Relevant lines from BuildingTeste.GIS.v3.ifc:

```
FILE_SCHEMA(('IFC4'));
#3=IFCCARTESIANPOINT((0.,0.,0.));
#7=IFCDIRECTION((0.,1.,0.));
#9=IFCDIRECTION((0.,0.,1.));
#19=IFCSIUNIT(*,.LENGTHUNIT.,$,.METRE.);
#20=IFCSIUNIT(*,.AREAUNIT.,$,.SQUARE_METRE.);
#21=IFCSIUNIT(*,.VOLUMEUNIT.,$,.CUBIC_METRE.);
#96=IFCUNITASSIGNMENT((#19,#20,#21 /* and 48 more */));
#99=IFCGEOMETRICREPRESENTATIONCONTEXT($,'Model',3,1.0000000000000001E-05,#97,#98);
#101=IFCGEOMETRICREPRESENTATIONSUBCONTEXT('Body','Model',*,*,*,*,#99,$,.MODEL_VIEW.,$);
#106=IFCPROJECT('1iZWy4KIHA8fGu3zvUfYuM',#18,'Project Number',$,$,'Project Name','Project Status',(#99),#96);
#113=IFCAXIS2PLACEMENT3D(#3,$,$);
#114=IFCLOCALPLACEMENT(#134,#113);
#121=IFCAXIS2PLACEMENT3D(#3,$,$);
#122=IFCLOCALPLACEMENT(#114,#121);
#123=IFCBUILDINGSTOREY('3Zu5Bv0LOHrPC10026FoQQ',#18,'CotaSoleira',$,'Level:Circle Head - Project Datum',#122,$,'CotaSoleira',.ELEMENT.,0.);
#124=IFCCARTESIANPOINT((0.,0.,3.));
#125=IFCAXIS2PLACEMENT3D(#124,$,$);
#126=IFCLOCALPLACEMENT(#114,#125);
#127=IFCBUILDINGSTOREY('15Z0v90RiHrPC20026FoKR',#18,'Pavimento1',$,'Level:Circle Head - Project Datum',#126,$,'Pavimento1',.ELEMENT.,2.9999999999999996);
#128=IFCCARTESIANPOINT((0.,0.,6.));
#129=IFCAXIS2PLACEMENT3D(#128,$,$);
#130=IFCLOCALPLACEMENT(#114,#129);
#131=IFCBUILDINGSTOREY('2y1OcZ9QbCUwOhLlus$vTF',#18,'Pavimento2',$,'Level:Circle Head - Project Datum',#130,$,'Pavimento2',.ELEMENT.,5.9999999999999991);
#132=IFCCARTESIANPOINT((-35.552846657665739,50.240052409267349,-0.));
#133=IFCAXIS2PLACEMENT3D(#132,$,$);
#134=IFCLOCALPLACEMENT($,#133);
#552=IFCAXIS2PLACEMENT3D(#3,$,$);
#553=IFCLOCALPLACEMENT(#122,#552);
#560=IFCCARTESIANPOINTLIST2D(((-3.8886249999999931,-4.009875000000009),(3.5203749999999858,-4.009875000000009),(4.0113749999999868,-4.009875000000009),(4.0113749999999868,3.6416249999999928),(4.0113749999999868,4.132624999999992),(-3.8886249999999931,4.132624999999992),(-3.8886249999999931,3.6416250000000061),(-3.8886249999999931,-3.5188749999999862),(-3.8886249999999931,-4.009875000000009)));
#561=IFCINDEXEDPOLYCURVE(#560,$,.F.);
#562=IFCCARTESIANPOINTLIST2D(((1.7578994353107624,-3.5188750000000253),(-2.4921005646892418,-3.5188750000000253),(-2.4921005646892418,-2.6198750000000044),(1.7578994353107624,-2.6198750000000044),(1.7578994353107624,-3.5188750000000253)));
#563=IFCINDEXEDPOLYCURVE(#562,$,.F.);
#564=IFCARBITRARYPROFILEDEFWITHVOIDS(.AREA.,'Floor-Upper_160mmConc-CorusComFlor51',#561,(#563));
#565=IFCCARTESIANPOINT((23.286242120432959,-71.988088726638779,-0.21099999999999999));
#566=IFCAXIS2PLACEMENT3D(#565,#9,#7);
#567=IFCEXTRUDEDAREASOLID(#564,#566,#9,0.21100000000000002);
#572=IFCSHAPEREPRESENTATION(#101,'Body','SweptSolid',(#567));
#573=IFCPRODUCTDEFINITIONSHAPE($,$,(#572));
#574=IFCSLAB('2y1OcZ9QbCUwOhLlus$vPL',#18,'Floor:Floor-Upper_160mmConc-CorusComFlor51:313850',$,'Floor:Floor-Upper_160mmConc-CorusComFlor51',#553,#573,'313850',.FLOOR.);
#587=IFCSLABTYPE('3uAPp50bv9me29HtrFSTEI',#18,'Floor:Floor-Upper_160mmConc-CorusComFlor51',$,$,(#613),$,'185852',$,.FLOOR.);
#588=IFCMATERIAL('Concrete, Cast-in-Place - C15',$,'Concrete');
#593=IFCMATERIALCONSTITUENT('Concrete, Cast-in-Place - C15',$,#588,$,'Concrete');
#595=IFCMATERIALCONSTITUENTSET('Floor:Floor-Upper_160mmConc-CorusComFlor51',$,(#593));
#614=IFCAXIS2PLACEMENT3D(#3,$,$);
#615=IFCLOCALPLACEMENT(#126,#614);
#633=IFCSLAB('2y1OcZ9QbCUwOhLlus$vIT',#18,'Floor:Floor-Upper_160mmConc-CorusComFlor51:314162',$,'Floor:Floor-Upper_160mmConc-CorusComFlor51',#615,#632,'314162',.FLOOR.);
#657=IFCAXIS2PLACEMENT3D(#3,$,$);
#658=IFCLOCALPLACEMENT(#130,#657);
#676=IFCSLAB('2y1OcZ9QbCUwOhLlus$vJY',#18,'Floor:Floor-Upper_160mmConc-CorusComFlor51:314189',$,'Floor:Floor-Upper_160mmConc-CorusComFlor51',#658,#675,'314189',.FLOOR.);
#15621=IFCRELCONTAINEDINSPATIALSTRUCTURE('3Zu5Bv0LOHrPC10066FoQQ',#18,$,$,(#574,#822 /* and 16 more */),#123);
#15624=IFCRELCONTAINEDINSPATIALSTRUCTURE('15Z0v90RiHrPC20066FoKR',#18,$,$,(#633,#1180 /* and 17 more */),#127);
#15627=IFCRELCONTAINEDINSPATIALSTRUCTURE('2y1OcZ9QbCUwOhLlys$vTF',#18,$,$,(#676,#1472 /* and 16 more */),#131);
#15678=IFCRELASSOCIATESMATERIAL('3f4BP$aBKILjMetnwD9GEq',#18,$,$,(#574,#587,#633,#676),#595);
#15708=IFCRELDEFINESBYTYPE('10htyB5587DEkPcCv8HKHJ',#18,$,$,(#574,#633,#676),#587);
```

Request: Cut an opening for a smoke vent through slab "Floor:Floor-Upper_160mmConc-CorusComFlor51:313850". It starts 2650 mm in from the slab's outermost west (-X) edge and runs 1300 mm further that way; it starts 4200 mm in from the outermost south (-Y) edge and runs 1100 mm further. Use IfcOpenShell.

```python
import numpy as np
import ifcopenshell
import ifcopenshell.api.feature
import ifcopenshell.api.geometry
import ifcopenshell.api.root
import ifcopenshell.geom
import ifcopenshell.util.placement
import ifcopenshell.util.representation
import ifcopenshell.util.shape
import ifcopenshell.util.unit

model = ifcopenshell.open("BuildingTeste.GIS.v3.ifc")
unit_scale = ifcopenshell.util.unit.calculate_unit_scale(model)
settings = ifcopenshell.geom.settings()


def volume(element):
    """Net volume in cubic metres, openings subtracted."""
    shape = ifcopenshell.geom.create_shape(settings, element)
    return ifcopenshell.util.shape.get_volume(shape.geometry)


slab = model.by_id(574)
before = volume(slab)

# Extent in the slab's own axes, in metres. The edges named are its -X and -Y sides.
slab_shape = ifcopenshell.geom.create_shape(settings, slab)
vertices = ifcopenshell.util.shape.get_vertices(slab_shape.geometry)
x_min, y_min, bottom = vertices.min(axis=0)
top = vertices[:, 2].max()

opening = ifcopenshell.api.root.create_entity(model, ifc_class="IfcOpeningElement", name="Smoke vent opening", predefined_type="OPENING")
context = ifcopenshell.util.representation.get_context(model, "Model", "Body", "MODEL_VIEW")
width, depth = 1.3, 1.1
outline = [(0.0, 0.0), (width, 0.0), (width, depth), (0.0, depth), (0.0, 0.0)]
# Overshoot both faces by 50 mm so the cut is clean.
shape = ifcopenshell.api.geometry.add_slab_representation(
    model, context=context, depth=top - bottom + 0.1, polyline=outline
)
ifcopenshell.api.geometry.assign_representation(model, product=opening, representation=shape)

matrix = ifcopenshell.util.placement.get_local_placement(slab.ObjectPlacement)
matrix[:, 3] = matrix @ np.append(np.array([x_min + 2.65, y_min + 4.2, bottom - 0.05]) / unit_scale, 1.0)
ifcopenshell.api.geometry.edit_object_placement(model, product=opening, matrix=matrix, is_si=False)
ifcopenshell.api.feature.add_feature(model, feature=opening, element=slab)

after = volume(slab)

print(f"slab volume {before:.3f} -> {after:.3f} m3")

model.write("BuildingTeste.GIS.v3_v2.ifc")
```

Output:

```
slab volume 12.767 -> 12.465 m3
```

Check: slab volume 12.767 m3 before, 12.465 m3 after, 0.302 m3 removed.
